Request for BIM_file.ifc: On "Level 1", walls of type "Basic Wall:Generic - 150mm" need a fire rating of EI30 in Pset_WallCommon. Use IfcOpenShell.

First a look at what the model holds.

```python
import ifcopenshell
import ifcopenshell.util.element

model = ifcopenshell.open("BIM_file.ifc")
print(model.schema)
storey = next(s for s in model.by_type("IfcBuildingStorey") if s.Name == "Level 1")
walls = [e for e in ifcopenshell.util.element.get_decomposition(storey) if e.is_a("IfcWall")]
seen = {}
for e in walls:
    element_type = ifcopenshell.util.element.get_type(e)
    key = (element_type.Name if element_type != e and element_type else None, ifcopenshell.util.element.get_pset(e, "Pset_WallCommon", "FireRating"))
    seen[key] = seen.get(key, 0) + 1
for (name, value), count in sorted(seen.items(), key=str):
    print(count, "x", name, "|", value)
```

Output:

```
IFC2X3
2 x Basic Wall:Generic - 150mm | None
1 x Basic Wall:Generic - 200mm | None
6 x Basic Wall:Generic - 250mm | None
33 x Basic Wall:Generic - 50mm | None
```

```python
import ifcopenshell
import ifcopenshell.api.pset
import ifcopenshell.util.element

model = ifcopenshell.open("BIM_file.ifc")

storey = next(s for s in model.by_type("IfcBuildingStorey") if s.Name == "Level 1")
walls = [e for e in ifcopenshell.util.element.get_decomposition(storey) if e.is_a("IfcWall")]

count = 0
for e in walls:
    element_type = ifcopenshell.util.element.get_type(e)
    if element_type in (None, e) or element_type.Name != "Basic Wall:Generic - 150mm":
        continue
    # add_pset returns the element's existing set when there is one.
    pset = ifcopenshell.api.pset.add_pset(model, product=e, name="Pset_WallCommon")
    ifcopenshell.api.pset.edit_pset(model, pset=pset, properties={"FireRating": "EI30"})
    count += 1

print(count, "walls updated")

model.write("BIM_file-out.ifc")
```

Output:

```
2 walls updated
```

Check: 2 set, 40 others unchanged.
